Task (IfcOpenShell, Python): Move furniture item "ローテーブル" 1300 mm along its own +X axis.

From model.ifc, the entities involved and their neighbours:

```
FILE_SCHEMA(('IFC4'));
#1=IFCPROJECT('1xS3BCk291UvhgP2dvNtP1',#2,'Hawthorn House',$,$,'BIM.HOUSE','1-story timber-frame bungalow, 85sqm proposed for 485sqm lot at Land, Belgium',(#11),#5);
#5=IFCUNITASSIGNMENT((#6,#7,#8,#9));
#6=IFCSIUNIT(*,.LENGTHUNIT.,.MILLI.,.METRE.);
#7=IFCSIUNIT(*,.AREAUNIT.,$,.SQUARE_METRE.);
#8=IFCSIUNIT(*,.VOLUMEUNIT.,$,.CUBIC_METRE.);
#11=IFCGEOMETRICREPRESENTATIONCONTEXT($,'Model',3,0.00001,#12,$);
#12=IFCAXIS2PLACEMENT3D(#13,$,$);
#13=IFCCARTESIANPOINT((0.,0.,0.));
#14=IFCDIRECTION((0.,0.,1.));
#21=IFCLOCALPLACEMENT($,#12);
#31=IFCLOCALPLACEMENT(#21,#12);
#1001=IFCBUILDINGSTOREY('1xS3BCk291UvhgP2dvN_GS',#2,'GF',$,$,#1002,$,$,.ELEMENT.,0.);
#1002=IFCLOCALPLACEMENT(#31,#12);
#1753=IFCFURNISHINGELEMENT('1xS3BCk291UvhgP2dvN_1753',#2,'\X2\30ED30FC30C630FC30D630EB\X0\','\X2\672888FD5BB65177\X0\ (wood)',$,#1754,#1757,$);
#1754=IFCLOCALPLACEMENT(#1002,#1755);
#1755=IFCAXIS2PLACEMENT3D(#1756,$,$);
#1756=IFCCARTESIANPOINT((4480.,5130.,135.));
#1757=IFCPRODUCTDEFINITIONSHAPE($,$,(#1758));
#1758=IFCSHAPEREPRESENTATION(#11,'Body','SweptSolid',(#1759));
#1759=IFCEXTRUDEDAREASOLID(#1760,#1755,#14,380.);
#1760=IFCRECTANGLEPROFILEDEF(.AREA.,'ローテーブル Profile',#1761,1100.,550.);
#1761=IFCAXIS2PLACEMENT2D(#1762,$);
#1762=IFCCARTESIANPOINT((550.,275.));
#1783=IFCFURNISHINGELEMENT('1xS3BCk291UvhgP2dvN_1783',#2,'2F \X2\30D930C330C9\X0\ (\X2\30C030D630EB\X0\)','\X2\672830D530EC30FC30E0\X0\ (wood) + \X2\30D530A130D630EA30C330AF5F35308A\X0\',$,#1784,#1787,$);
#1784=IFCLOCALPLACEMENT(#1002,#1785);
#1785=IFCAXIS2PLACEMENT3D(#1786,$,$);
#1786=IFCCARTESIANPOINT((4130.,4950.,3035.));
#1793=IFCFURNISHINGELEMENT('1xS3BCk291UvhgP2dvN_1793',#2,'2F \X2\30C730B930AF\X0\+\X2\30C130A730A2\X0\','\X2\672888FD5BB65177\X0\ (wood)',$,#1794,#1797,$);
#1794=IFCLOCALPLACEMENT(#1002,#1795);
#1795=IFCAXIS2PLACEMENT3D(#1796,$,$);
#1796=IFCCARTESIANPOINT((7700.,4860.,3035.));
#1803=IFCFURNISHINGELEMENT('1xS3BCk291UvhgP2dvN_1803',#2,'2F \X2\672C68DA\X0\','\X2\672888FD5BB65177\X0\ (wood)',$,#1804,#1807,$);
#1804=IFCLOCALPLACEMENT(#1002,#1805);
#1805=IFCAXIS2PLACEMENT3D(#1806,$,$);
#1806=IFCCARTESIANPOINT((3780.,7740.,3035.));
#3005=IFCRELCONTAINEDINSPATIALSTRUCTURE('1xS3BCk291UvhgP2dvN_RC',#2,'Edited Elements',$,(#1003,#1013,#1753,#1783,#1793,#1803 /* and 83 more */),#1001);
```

```python
import ifcopenshell
import ifcopenshell.api.geometry
import ifcopenshell.util.placement

model = ifcopenshell.open("model.ifc")

item = model.by_id(1753)
matrix = ifcopenshell.util.placement.get_local_placement(item.ObjectPlacement)
matrix[:3, 3] += matrix[:3, 0] * 1300.0
ifcopenshell.api.geometry.edit_object_placement(model, product=item, matrix=matrix, is_si=False)

print(ifcopenshell.util.placement.get_local_placement(item.ObjectPlacement).round(3) + 0.0)

model.write("model_rev.ifc")
```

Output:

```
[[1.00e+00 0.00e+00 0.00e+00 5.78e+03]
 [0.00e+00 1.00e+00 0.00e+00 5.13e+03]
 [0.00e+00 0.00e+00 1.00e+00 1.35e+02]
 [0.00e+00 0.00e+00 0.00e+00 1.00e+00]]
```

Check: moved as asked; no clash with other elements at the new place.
